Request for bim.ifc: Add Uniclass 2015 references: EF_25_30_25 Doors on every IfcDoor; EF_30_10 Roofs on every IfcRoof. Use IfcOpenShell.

First a look at what the model holds.

```python
import ifcopenshell

model = ifcopenshell.open("bim.ifc")
print(model.schema)
print("classifications:", [c.Name for c in model.by_type("IfcClassification")])
for ifc_class in ("IfcDoor", "IfcRoof", "IfcStair", "IfcWall", "IfcWindow"):
    print(ifc_class, len(model.by_type(ifc_class)))
```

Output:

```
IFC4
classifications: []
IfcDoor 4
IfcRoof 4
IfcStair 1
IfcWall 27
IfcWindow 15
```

```python
import ifcopenshell
import ifcopenshell.api.classification

model = ifcopenshell.open("bim.ifc")

system = ifcopenshell.api.classification.add_classification(model, classification="Uniclass 2015")

codes = {
    "IfcDoor": ("EF_25_30_25", "Doors"),
    "IfcRoof": ("EF_30_10", "Roofs"),
}
for ifc_class, (code, name) in codes.items():
    products = model.by_type(ifc_class)
    ifcopenshell.api.classification.add_reference(
        model, products=products, classification=system, identification=code, name=name
    )
    print(code, len(products))

model.write("bim_edited.ifc")
```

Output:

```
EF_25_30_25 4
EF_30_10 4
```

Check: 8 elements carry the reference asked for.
